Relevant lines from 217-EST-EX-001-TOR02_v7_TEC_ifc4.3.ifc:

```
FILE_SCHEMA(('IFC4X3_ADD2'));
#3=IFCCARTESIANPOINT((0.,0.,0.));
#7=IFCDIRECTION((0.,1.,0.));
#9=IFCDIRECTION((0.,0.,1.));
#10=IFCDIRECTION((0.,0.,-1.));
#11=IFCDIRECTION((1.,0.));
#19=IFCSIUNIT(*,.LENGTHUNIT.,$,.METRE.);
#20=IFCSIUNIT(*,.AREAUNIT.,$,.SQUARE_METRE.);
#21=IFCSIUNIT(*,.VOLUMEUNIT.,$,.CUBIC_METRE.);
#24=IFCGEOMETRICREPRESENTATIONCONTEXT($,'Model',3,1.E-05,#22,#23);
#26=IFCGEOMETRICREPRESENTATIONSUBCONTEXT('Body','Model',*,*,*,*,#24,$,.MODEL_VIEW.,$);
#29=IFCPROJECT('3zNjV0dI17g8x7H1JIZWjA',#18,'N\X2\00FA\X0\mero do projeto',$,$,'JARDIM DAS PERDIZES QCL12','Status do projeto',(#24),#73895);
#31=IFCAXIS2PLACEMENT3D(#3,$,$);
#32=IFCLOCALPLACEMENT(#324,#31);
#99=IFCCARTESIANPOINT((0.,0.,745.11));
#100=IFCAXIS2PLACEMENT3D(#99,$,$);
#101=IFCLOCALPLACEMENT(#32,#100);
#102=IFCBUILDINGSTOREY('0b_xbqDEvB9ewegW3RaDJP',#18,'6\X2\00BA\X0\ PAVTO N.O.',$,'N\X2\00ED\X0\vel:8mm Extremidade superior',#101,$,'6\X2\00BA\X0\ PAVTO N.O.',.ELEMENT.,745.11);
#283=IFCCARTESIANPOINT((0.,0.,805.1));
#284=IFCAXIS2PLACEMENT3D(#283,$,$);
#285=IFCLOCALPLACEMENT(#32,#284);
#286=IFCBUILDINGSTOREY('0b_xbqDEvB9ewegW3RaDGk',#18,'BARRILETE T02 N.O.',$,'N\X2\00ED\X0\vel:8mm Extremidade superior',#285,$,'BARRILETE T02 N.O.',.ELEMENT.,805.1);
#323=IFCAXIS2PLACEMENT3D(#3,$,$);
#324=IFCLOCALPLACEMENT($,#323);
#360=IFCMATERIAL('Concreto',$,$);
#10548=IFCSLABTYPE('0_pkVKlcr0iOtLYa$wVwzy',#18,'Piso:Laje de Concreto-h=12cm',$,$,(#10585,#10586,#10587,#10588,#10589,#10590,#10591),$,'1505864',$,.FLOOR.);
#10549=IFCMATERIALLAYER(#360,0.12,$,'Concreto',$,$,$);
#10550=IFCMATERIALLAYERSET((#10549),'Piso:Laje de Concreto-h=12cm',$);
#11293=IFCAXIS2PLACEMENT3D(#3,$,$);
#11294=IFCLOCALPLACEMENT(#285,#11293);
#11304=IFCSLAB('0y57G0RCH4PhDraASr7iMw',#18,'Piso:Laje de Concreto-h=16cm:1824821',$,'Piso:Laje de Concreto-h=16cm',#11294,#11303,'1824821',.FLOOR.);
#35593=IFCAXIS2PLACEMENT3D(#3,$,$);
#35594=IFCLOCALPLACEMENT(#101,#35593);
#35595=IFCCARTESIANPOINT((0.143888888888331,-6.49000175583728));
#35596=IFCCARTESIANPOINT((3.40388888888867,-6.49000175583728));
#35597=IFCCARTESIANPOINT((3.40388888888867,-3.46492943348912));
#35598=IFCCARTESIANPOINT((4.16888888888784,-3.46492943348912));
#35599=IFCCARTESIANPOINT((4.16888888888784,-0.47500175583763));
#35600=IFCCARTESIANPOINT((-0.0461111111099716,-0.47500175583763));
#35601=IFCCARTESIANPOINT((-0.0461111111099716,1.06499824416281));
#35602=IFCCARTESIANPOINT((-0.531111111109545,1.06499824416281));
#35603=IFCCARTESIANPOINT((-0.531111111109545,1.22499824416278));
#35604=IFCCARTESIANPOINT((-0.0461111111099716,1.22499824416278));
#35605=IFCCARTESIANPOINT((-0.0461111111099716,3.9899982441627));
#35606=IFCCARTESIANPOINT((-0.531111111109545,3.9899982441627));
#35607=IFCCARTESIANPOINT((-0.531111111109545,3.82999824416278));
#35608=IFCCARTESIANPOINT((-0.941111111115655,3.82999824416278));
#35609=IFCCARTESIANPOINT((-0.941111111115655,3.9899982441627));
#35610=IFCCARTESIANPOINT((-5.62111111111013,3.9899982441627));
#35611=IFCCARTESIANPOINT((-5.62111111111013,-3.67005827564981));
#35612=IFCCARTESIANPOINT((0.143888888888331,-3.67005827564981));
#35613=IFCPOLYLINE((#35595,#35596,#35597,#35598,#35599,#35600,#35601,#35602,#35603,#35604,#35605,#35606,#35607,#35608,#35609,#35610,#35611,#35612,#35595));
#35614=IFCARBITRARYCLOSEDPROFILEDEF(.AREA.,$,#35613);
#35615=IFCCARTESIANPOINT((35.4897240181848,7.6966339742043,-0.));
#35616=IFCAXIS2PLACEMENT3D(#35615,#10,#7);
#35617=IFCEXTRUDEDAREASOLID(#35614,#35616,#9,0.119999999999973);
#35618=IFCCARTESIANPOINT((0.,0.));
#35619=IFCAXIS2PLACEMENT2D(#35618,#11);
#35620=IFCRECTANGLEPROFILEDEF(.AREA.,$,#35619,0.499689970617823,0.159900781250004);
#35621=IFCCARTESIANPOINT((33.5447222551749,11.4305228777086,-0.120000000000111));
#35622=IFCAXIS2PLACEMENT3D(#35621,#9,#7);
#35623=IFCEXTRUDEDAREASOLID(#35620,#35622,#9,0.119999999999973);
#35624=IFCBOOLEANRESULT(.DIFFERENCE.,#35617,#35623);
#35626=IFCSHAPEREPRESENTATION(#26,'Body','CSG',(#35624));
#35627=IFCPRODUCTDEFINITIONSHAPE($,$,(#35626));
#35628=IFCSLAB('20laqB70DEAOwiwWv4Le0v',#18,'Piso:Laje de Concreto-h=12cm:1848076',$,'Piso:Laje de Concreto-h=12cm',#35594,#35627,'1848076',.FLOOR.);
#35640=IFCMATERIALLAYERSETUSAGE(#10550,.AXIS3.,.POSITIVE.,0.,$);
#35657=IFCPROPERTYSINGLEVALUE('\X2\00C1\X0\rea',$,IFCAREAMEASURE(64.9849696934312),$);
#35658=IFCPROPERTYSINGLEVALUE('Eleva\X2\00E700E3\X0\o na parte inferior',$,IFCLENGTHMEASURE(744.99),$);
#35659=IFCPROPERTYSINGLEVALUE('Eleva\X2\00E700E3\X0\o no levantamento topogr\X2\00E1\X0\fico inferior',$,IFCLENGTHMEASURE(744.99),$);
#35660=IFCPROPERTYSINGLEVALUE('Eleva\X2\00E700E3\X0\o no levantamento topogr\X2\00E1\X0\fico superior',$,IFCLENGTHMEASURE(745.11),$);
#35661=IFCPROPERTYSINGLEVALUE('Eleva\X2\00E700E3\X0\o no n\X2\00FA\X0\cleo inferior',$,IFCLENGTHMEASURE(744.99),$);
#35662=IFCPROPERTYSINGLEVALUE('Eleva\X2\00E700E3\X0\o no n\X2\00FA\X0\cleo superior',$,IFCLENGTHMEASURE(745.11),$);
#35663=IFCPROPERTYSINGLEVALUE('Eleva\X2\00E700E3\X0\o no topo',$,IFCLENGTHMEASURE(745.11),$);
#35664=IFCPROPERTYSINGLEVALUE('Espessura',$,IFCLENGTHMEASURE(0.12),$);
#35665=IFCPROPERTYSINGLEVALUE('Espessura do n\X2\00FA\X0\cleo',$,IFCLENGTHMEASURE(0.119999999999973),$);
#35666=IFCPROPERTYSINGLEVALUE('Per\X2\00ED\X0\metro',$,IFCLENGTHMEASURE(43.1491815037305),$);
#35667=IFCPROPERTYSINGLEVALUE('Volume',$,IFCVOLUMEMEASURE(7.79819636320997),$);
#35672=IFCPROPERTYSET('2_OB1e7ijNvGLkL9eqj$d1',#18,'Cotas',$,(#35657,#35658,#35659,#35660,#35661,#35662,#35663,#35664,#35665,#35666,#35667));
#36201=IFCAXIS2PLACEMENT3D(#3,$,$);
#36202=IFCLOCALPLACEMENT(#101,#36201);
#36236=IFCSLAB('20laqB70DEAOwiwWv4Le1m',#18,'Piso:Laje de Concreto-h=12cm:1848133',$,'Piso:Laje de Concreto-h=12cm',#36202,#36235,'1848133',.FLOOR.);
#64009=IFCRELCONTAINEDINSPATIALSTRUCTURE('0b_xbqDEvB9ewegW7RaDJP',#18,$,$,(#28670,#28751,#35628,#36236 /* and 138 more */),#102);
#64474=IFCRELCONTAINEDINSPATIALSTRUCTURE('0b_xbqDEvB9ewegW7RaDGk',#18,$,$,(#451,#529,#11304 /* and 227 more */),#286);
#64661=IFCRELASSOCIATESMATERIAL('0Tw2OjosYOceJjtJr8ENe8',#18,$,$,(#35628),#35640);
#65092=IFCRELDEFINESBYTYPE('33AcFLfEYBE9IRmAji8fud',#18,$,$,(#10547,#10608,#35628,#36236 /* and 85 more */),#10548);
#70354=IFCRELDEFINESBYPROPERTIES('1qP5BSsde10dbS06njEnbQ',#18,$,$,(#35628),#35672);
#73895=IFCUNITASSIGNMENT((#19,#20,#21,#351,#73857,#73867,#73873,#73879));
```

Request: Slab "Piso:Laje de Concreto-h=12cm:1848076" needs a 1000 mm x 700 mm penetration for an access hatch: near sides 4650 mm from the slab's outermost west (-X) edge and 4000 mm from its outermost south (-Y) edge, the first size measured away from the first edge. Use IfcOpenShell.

```python
import numpy as np
import ifcopenshell
import ifcopenshell.api.feature
import ifcopenshell.api.geometry
import ifcopenshell.api.pset
import ifcopenshell.api.root
import ifcopenshell.geom
import ifcopenshell.util.element
import ifcopenshell.util.placement
import ifcopenshell.util.representation
import ifcopenshell.util.shape
import ifcopenshell.util.unit

model = ifcopenshell.open("217-EST-EX-001-TOR02_v7_TEC_ifc4.3.ifc")
unit_scale = ifcopenshell.util.unit.calculate_unit_scale(model)
area_scale = ifcopenshell.util.unit.calculate_unit_scale(model, "AREAUNIT")
volume_scale = ifcopenshell.util.unit.calculate_unit_scale(model, "VOLUMEUNIT")
settings = ifcopenshell.geom.settings()


def volume(element):
    """Net volume in cubic metres, openings subtracted."""
    shape = ifcopenshell.geom.create_shape(settings, element)
    return ifcopenshell.util.shape.get_volume(shape.geometry)


slab = model.by_id(35628)
before = volume(slab)

# Extent in the slab's own axes, in metres. The edges named are its -X and -Y sides.
slab_shape = ifcopenshell.geom.create_shape(settings, slab)
vertices = ifcopenshell.util.shape.get_vertices(slab_shape.geometry)
x_min, y_min, bottom = vertices.min(axis=0)
top = vertices[:, 2].max()

opening = ifcopenshell.api.root.create_entity(model, ifc_class="IfcOpeningElement", name="Access hatch opening", predefined_type="OPENING")
context = ifcopenshell.util.representation.get_context(model, "Model", "Body", "MODEL_VIEW")
width, depth = 1, 0.7
outline = [(0.0, 0.0), (width, 0.0), (width, depth), (0.0, depth), (0.0, 0.0)]
# Overshoot both faces by 50 mm so the cut is clean.
shape = ifcopenshell.api.geometry.add_slab_representation(
    model, context=context, depth=top - bottom + 0.1, polyline=outline
)
ifcopenshell.api.geometry.assign_representation(model, product=opening, representation=shape)

matrix = ifcopenshell.util.placement.get_local_placement(slab.ObjectPlacement)
matrix[:, 3] = matrix @ np.append(np.array([x_min + 4.65, y_min + 4, bottom - 0.05]) / unit_scale, 1.0)
ifcopenshell.api.geometry.edit_object_placement(model, product=opening, matrix=matrix, is_si=False)
ifcopenshell.api.feature.add_feature(model, feature=opening, element=slab)

after = volume(slab)

# Update the slab's stored quantities.
pset = model.by_id(ifcopenshell.util.element.get_pset(slab, "Cotas", should_inherit=False)["id"])
ifcopenshell.api.pset.edit_pset(model, pset=pset, properties={
    "Área": model.create_entity("IfcAreaMeasure", after / (top - bottom) / area_scale),
    "Volume": model.create_entity("IfcVolumeMeasure", after / volume_scale),
})

print(f"slab volume {before:.3f} -> {after:.3f} m3")

model.write("217-EST-EX-001-TOR02_v7_TEC_ifc4.3_updated.ifc")
```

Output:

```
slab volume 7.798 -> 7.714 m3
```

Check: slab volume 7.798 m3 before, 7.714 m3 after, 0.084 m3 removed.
